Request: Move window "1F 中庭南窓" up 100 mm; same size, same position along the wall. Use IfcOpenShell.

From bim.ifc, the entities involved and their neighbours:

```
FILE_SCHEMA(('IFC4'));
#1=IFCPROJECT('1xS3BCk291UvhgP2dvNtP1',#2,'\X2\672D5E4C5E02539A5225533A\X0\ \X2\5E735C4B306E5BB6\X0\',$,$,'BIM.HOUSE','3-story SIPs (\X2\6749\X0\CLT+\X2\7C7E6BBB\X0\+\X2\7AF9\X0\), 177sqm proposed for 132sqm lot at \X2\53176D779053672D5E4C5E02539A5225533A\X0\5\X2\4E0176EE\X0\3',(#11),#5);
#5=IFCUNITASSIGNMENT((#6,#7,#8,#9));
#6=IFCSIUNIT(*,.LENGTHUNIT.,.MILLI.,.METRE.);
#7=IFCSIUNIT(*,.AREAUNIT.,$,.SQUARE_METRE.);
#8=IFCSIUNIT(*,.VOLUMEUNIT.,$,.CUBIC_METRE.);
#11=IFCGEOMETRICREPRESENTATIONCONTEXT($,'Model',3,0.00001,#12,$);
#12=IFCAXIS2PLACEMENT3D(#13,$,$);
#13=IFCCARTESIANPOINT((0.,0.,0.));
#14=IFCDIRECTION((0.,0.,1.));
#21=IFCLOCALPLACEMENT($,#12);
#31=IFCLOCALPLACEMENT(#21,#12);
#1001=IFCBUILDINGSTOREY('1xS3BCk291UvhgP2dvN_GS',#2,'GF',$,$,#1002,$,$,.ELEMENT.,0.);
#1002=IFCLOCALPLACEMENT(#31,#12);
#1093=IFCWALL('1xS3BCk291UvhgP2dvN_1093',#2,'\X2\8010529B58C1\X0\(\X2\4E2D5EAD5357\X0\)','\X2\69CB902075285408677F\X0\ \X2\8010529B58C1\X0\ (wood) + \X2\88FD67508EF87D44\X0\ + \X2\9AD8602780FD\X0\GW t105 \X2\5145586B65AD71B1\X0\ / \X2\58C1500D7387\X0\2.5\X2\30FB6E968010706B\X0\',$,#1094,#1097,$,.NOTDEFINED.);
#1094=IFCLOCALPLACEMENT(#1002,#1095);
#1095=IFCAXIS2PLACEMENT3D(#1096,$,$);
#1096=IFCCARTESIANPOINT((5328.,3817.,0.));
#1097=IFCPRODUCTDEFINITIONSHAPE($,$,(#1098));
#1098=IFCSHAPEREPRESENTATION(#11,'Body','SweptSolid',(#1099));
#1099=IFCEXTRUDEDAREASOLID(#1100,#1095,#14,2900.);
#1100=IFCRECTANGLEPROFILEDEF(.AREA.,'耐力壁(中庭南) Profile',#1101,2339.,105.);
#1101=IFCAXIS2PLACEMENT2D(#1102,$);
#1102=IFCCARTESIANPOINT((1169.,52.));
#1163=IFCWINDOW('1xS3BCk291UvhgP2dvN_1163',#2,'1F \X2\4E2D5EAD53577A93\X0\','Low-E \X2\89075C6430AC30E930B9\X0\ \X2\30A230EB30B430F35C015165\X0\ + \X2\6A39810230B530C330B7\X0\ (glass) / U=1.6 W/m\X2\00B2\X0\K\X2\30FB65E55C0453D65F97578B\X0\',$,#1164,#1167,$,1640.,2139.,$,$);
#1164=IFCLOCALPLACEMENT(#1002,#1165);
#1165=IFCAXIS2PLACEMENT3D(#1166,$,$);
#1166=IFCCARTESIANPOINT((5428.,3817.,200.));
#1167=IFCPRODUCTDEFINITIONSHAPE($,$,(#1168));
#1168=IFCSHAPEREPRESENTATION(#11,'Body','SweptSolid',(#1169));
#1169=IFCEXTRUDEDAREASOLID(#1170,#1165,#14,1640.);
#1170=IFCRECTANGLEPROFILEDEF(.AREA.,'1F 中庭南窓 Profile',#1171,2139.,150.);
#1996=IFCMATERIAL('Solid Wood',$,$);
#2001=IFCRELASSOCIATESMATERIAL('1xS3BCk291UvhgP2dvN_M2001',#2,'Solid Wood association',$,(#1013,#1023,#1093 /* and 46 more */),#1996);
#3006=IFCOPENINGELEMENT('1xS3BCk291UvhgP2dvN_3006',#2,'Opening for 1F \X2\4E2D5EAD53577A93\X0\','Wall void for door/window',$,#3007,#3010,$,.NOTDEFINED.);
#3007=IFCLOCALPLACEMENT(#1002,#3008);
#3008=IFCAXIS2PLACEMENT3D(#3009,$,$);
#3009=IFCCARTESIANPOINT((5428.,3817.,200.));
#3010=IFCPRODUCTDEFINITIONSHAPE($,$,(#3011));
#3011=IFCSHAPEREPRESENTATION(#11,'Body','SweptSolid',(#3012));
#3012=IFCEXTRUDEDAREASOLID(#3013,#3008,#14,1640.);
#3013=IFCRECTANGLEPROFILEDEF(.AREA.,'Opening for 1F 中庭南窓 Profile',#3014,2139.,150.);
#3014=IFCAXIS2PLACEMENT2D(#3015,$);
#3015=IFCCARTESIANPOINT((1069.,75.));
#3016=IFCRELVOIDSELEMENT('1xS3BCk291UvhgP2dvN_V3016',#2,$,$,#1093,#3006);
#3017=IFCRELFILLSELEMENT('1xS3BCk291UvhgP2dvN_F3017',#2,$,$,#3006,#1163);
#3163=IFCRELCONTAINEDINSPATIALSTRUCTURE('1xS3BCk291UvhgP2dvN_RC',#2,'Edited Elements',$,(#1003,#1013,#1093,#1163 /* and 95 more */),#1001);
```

```python
import numpy as np
import ifcopenshell
import ifcopenshell.api.geometry
import ifcopenshell.util.placement
import ifcopenshell.util.unit

model = ifcopenshell.open("bim.ifc")
unit_scale = ifcopenshell.util.unit.calculate_unit_scale(model)

window = model.by_guid("1xS3BCk291UvhgP2dvN_1163")
opening = window.FillsVoids[0].RelatingOpeningElement
dz = 0.1 / unit_scale

shift = np.array([0.0, 0.0, dz])
# The window is not placed relative to its opening, so move both.
for product in (opening, window):
    matrix = ifcopenshell.util.placement.get_local_placement(product.ObjectPlacement)
    matrix[:3, 3] += shift
    ifcopenshell.api.geometry.edit_object_placement(model, product=product, matrix=matrix, is_si=False)

print(f"moved by {dz * unit_scale:+.3f} m")

model.write("bim_v2.ifc")
```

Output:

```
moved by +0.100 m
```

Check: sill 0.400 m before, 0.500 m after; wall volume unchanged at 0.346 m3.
